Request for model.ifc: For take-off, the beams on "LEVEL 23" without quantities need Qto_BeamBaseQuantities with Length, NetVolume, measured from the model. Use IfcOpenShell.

First a look at what the model holds.

```python
import ifcopenshell
import ifcopenshell.util.element
import ifcopenshell.util.unit

model = ifcopenshell.open("model.ifc")
print(model.schema)
for unit_type in ("LENGTHUNIT", "AREAUNIT", "VOLUMEUNIT"):
    print(unit_type, ifcopenshell.util.unit.calculate_unit_scale(model, unit_type))
storey = next(s for s in model.by_type("IfcBuildingStorey") if s.Name == "LEVEL 23")
beams = [e for e in ifcopenshell.util.element.get_decomposition(storey) if e.is_a("IfcBeam")]
for e in sorted(beams, key=lambda e: e.id()):
    print(e.id(), e.is_a(), e.Name, list(ifcopenshell.util.element.get_psets(e, qtos_only=True)), sep=" | ")
```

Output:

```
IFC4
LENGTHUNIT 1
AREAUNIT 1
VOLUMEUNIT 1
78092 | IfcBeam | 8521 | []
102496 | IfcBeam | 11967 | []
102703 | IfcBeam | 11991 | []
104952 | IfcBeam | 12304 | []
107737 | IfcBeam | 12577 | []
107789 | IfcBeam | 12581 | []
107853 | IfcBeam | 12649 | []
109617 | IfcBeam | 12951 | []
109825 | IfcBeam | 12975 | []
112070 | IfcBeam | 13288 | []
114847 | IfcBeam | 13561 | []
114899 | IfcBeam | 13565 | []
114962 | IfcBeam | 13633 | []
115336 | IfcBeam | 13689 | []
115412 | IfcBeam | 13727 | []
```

```python
import ifcopenshell
import ifcopenshell.api.pset
import ifcopenshell.geom
import ifcopenshell.util.element
import ifcopenshell.util.shape
import ifcopenshell.util.unit

model = ifcopenshell.open("model.ifc")
unit_scale = ifcopenshell.util.unit.calculate_unit_scale(model)
volume_scale = ifcopenshell.util.unit.calculate_unit_scale(model, "VOLUMEUNIT")
settings = ifcopenshell.geom.settings()

storey = next(s for s in model.by_type("IfcBuildingStorey") if s.Name == "LEVEL 23")
beams = [e for e in ifcopenshell.util.element.get_decomposition(storey) if e.is_a("IfcBeam")]

for e in sorted(beams, key=lambda e: e.id()):
    if ifcopenshell.util.element.get_psets(e, qtos_only=True, should_inherit=False):
        continue
    # Geometry comes back in metres, in the element's own axes.
    shape = ifcopenshell.geom.create_shape(settings, e)
    values = {
        "Length": ifcopenshell.util.shape.get_max_xyz(shape.geometry) / unit_scale,
        "NetVolume": ifcopenshell.util.shape.get_volume(shape.geometry) / volume_scale,
    }
    qto = ifcopenshell.api.pset.add_qto(model, product=e, name="Qto_BeamBaseQuantities")
    ifcopenshell.api.pset.edit_qto(model, qto=qto, properties=values)
    print(e.id(), {k: round(v, 3) for k, v in values.items()})

model.write("model_updated.ifc")
```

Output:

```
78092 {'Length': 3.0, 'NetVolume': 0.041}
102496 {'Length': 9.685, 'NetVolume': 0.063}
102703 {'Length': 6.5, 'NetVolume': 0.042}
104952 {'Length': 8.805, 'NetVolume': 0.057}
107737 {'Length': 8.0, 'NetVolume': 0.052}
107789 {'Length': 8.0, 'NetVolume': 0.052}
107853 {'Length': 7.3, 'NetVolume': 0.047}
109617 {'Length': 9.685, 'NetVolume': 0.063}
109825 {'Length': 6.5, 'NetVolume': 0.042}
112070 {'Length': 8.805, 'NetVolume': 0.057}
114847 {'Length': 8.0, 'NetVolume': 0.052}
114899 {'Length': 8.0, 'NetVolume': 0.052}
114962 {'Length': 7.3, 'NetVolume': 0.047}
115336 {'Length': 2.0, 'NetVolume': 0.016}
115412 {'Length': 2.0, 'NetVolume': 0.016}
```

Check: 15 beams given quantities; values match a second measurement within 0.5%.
